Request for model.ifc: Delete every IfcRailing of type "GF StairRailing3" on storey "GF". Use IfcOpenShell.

First a look at what the model holds.

```python
import ifcopenshell
import ifcopenshell.util.element

model = ifcopenshell.open("model.ifc")
print(model.schema)
storey = next(s for s in model.by_type("IfcBuildingStorey") if s.Name == "GF")
railings = [e for e in ifcopenshell.util.element.get_decomposition(storey) if e.is_a("IfcRailing")]
seen = {}
for e in railings:
    element_type = ifcopenshell.util.element.get_type(e)
    name = element_type.Name if element_type not in (None, e) else None
    seen[name] = seen.get(name, 0) + 1
for name, count in sorted(seen.items(), key=str):
    print(count, "x", name)
```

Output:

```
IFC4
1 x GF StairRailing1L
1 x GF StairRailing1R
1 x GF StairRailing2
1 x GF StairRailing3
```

```python
import ifcopenshell
import ifcopenshell.api.root
import ifcopenshell.util.element

model = ifcopenshell.open("model.ifc")

storey = next(s for s in model.by_type("IfcBuildingStorey") if s.Name == "GF")
railings = [e for e in ifcopenshell.util.element.get_decomposition(storey) if e.is_a("IfcRailing")]
targets = [e for e in railings if (t := ifcopenshell.util.element.get_type(e)) not in (None, e) and t.Name == "GF StairRailing3"]

for e in targets:
    ifcopenshell.api.root.remove_product(model, product=e)
print(len(targets), "removed")

model.write("model_edited.ifc")
```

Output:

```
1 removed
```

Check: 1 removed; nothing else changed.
